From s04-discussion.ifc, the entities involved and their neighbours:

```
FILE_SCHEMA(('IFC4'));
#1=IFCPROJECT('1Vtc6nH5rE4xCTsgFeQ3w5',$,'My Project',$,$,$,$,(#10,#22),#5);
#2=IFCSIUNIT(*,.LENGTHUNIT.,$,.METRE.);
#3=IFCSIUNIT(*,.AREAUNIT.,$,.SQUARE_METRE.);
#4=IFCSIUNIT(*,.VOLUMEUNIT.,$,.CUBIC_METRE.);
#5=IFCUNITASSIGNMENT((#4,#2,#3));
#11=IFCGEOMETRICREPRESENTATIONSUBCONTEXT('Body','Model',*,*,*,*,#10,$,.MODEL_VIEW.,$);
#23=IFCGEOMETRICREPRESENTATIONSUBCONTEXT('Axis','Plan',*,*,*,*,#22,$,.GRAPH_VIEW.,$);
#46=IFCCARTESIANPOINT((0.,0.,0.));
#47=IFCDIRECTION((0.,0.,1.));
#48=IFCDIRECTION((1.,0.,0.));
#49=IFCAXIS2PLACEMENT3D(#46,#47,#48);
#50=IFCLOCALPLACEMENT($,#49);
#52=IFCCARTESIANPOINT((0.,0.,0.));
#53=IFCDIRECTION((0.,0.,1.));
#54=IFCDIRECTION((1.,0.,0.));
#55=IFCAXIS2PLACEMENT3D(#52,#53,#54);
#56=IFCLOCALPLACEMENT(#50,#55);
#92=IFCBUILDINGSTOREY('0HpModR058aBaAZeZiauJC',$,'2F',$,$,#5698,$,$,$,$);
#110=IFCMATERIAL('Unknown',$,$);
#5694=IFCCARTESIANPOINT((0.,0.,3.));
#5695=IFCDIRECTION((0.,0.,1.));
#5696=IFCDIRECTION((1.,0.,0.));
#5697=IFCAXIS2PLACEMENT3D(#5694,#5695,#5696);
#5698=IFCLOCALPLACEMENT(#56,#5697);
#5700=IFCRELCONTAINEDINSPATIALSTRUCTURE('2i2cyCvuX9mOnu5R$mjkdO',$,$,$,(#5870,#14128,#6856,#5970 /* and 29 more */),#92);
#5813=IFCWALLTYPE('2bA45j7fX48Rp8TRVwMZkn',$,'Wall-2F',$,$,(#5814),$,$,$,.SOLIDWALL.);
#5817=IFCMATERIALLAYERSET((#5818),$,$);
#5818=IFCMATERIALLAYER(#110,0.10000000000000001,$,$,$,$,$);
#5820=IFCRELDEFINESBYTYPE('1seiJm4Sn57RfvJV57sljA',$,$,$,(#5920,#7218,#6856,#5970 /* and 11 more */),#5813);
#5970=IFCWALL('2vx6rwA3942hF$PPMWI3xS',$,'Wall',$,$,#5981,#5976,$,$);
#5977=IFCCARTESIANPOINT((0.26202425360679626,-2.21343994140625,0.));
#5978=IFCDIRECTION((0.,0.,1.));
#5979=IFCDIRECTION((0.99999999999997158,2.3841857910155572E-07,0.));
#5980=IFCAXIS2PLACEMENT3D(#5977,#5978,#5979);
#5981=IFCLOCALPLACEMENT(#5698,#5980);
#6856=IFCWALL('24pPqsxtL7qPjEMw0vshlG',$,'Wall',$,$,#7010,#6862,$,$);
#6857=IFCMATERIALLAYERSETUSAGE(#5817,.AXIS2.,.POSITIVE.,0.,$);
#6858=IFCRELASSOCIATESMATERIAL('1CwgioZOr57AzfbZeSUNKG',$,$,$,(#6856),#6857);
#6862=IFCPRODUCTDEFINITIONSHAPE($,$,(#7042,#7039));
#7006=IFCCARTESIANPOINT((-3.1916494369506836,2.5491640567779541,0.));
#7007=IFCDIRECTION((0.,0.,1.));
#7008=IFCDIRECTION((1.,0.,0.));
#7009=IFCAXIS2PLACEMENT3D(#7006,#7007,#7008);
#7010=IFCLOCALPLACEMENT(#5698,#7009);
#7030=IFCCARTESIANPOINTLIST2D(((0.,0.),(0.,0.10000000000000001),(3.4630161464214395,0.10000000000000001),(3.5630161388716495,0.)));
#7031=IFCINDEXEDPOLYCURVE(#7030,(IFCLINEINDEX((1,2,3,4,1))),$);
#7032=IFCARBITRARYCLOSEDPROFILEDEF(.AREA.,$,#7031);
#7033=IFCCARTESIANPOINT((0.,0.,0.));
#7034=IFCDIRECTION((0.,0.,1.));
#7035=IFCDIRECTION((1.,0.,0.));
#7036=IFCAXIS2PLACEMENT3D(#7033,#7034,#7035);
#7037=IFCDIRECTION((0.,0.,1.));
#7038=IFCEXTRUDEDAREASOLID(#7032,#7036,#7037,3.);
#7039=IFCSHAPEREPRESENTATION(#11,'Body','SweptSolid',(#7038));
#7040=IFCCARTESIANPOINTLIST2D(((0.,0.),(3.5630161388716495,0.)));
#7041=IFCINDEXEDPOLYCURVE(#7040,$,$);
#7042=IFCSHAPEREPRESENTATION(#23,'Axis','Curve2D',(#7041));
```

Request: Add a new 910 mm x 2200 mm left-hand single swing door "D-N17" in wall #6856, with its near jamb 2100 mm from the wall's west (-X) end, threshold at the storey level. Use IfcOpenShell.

```python
import numpy as np
import ifcopenshell
import ifcopenshell.api.feature
import ifcopenshell.api.geometry
import ifcopenshell.api.root
import ifcopenshell.api.spatial
import ifcopenshell.geom
import ifcopenshell.util.element
import ifcopenshell.util.placement
import ifcopenshell.util.representation
import ifcopenshell.util.shape
import ifcopenshell.util.unit

model = ifcopenshell.open("s04-discussion.ifc")
unit_scale = ifcopenshell.util.unit.calculate_unit_scale(model)
settings = ifcopenshell.geom.settings()


def volume(element):
    """Net volume in cubic metres, openings subtracted."""
    shape = ifcopenshell.geom.create_shape(settings, element)
    return ifcopenshell.util.shape.get_volume(shape.geometry)


wall = model.by_guid("24pPqsxtL7qPjEMw0vshlG")
storey = ifcopenshell.util.element.get_container(wall, ifc_class="IfcBuildingStorey")
context = ifcopenshell.util.representation.get_context(model, "Model", "Body", "MODEL_VIEW")
before = volume(wall)

width, height, from_end, sill = 0.91, 2.2, 2.1, 0.0  # metres

# The wall runs along its own X axis, and the end named is its -X end.
wall_shape = ifcopenshell.geom.create_shape(settings, wall)
x, y, z = ifcopenshell.util.shape.get_vertices(wall_shape.geometry).T
start = x.min() + from_end
face, thickness = float(y.min()), float(y.max() - y.min())
wall_matrix = ifcopenshell.util.placement.get_local_placement(wall.ObjectPlacement)
level = ifcopenshell.util.placement.get_local_placement(storey.ObjectPlacement)[2, 3]


def in_wall(x, y):
    """Placement at x, y metres in the wall's axes, at sill height."""
    matrix = wall_matrix.copy()
    matrix[:, 3] = wall_matrix @ np.array([x / unit_scale, y / unit_scale, 0.0, 1.0])
    matrix[2, 3] = level + sill / unit_scale
    return matrix


# Opening: a box that overshoots both wall faces by 50 mm.
opening = ifcopenshell.api.root.create_entity(model, ifc_class="IfcOpeningElement", predefined_type="OPENING")
box = ifcopenshell.api.geometry.add_wall_representation(
    model, context=context, length=width, height=height, thickness=thickness + 0.1
)
ifcopenshell.api.geometry.assign_representation(model, product=opening, representation=box)
ifcopenshell.api.geometry.edit_object_placement(model, product=opening, matrix=in_wall(start, face - 0.05), is_si=False)
ifcopenshell.api.feature.add_feature(model, feature=opening, element=wall)

door = ifcopenshell.api.root.create_entity(model, ifc_class="IfcDoor", name="D-N17", predefined_type="DOOR")
door.OverallWidth, door.OverallHeight = width / unit_scale, height / unit_scale
door.OperationType = "SINGLE_SWING_LEFT"
body = ifcopenshell.api.geometry.add_door_representation(
    model,
    context=context,
    overall_width=door.OverallWidth,
    overall_height=door.OverallHeight,
    operation_type="SINGLE_SWING_LEFT",
    lining_properties={"LiningDepth": thickness / unit_scale, "ThresholdDepth": thickness / unit_scale},
)
ifcopenshell.api.geometry.assign_representation(model, product=door, representation=body)
ifcopenshell.api.spatial.assign_container(model, products=[door], relating_structure=storey)
ifcopenshell.api.feature.add_filling(model, opening=opening, element=door)

# The lining spans the wall, so the door starts at the wall face.
ifcopenshell.api.geometry.edit_object_placement(model, product=door, matrix=in_wall(start, face), is_si=False)

after = volume(wall)

print(f"wall volume {before:.3f} -> {after:.3f} m3")

model.write("s04-discussion_rev.ifc")
```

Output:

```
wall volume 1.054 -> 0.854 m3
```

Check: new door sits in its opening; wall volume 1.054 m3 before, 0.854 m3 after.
